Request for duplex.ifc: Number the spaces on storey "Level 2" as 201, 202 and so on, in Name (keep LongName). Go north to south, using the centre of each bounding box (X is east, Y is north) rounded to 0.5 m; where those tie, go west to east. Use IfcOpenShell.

First a look at what the model holds.

```python
import ifcopenshell
import ifcopenshell.util.element
import ifcopenshell.util.placement

model = ifcopenshell.open("duplex.ifc")
print(model.schema)
storey = next(s for s in model.by_type("IfcBuildingStorey") if s.Name == "Level 2")
spaces = [e for e in ifcopenshell.util.element.get_decomposition(storey) if e.is_a("IfcSpace")]
for e in sorted(spaces, key=lambda e: e.id()):
    origin = ifcopenshell.util.placement.get_local_placement(e.ObjectPlacement)[:3, 3]
    print(e.id(), e.Name, e.LongName, origin.round(2) + 0.0, sep=" | ")
```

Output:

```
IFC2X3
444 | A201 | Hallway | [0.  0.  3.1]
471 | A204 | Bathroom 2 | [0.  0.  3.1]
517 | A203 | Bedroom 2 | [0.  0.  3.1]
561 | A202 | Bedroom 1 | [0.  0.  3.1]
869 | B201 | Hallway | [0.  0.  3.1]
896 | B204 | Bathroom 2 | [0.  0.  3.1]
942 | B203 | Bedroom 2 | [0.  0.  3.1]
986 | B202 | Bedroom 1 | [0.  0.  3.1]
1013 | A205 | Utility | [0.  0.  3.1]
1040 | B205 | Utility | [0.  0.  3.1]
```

```python
import ifcopenshell
import ifcopenshell.geom
import ifcopenshell.util.element
import ifcopenshell.util.shape

model = ifcopenshell.open("duplex.ifc")
settings = ifcopenshell.geom.settings()
settings.set("use-world-coords", True)


def centre(element):
    shape = ifcopenshell.geom.create_shape(settings, element)
    return ifcopenshell.util.shape.get_bbox_centroid(shape.geometry)


storey = next(s for s in model.by_type("IfcBuildingStorey") if s.Name == "Level 2")
spaces = [e for e in ifcopenshell.util.element.get_decomposition(storey) if e.is_a("IfcSpace")]

# Insertion points can sit at a corner or the storey origin, so sort by the geometry (in metres).
centres = {e: centre(e) for e in spaces}
spaces.sort(key=lambda e: (-round(centres[e][1] / 0.5), centres[e][0]))

for i, e in enumerate(spaces, start=1):
    number = f"2{i:02d}"
    e.Name = number
    print(e.id(), number)

model.write("duplex_updated.ifc")
```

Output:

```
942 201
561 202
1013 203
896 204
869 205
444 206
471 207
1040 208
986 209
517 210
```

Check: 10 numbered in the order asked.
